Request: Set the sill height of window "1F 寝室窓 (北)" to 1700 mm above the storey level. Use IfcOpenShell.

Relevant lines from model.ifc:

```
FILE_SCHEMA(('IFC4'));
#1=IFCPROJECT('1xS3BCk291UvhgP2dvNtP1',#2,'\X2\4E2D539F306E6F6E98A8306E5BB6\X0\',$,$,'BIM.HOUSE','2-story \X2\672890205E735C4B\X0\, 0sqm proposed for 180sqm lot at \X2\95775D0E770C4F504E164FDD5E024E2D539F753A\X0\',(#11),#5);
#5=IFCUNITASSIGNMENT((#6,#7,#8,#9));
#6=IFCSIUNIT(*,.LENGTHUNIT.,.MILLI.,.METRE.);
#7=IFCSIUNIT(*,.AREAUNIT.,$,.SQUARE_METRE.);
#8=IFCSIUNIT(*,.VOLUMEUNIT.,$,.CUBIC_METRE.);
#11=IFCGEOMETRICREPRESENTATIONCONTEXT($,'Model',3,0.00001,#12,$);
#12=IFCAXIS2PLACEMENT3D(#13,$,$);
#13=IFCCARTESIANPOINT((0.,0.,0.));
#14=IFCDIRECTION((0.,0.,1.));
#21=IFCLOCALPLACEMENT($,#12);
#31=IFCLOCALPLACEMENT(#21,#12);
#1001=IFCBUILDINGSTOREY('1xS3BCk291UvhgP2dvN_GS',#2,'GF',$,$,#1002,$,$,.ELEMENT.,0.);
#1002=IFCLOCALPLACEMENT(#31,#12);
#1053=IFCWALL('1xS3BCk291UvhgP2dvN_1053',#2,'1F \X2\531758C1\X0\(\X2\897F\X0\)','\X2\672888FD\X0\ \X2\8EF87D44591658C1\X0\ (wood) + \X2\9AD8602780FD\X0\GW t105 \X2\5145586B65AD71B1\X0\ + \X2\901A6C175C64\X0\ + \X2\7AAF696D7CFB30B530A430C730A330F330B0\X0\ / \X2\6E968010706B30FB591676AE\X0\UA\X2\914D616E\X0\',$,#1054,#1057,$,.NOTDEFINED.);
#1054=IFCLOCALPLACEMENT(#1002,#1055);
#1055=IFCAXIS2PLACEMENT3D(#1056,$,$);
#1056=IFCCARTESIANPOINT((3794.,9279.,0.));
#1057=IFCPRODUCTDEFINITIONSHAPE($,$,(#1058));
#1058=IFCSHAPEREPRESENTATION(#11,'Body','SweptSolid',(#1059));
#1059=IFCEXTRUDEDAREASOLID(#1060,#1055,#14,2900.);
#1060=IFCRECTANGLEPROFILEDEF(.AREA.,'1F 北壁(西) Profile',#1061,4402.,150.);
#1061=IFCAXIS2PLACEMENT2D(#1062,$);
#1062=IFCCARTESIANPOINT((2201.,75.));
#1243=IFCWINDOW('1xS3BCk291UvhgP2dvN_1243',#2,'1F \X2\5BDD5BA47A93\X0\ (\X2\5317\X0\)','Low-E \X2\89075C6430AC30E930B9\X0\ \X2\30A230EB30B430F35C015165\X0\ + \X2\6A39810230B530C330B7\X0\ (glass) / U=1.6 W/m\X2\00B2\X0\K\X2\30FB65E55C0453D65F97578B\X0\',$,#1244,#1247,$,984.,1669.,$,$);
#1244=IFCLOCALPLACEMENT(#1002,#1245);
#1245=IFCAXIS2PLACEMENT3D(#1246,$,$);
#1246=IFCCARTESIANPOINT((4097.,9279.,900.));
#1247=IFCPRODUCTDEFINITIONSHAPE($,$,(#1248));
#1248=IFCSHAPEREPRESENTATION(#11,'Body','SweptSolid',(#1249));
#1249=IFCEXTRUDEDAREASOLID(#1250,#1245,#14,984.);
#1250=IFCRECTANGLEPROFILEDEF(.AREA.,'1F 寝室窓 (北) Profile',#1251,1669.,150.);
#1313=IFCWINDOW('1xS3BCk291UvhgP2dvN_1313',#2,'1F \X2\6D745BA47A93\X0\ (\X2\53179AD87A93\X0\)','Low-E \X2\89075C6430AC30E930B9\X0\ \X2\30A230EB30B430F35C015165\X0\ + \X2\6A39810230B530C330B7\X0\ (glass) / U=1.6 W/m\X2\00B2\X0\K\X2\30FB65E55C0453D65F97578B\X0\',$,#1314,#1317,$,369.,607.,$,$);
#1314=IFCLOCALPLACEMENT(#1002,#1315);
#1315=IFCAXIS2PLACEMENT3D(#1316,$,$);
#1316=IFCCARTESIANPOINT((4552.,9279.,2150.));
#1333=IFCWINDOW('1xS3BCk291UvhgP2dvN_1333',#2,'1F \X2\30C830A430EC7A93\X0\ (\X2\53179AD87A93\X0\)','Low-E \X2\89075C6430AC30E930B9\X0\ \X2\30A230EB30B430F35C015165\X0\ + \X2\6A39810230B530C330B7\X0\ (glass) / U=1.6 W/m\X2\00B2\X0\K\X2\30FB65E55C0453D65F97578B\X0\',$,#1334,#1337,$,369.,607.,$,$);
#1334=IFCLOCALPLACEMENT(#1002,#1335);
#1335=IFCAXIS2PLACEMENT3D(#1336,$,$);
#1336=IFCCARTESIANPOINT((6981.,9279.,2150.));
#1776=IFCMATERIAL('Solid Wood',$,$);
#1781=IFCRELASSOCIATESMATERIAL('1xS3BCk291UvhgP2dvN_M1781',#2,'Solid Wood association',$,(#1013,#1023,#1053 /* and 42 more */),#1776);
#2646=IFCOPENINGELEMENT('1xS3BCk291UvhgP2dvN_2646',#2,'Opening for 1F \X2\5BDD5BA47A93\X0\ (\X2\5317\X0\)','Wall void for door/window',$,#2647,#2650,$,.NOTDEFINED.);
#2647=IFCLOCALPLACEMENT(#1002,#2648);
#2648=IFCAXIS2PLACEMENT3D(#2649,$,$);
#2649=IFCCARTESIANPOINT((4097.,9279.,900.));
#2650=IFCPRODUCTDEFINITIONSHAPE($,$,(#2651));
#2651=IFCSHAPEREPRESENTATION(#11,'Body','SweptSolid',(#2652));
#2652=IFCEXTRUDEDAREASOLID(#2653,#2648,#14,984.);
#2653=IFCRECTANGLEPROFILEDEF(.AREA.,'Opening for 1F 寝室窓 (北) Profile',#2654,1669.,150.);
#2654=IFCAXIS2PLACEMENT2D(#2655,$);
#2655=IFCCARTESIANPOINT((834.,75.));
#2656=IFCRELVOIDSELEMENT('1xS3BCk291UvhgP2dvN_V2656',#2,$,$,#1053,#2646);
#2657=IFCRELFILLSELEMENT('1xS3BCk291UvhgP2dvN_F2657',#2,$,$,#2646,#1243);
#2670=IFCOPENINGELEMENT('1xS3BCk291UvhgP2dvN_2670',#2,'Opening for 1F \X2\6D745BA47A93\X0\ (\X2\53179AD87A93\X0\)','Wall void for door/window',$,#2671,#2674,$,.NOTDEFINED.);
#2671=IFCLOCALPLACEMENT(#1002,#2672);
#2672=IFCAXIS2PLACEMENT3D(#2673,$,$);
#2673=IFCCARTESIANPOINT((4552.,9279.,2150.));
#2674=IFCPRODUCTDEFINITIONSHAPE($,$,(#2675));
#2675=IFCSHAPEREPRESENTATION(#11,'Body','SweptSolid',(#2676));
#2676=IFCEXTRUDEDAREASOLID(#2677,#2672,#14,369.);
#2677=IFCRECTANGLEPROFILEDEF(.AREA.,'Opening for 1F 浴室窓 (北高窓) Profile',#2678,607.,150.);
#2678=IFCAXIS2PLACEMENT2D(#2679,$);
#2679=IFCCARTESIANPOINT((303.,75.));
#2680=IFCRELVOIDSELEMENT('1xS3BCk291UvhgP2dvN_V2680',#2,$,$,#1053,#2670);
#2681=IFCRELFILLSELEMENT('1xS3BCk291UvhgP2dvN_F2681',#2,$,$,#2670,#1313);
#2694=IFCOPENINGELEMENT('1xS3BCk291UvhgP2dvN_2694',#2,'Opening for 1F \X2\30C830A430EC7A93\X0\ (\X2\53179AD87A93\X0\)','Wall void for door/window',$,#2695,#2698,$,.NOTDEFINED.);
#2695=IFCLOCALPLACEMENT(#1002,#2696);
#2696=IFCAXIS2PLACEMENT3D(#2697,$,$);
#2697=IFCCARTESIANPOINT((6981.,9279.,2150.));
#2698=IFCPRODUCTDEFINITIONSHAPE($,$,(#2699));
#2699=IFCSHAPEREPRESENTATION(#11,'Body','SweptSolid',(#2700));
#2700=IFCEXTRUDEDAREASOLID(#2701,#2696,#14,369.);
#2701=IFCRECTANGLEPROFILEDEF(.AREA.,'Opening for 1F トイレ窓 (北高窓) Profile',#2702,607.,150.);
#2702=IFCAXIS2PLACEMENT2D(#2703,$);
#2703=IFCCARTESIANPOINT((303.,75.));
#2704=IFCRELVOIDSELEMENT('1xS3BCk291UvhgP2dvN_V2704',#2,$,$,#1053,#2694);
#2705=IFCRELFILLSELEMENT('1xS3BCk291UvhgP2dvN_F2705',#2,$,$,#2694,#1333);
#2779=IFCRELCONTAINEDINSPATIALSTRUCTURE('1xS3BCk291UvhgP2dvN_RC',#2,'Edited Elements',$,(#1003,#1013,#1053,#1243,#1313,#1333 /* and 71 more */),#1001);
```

```python
import numpy as np
import ifcopenshell
import ifcopenshell.api.geometry
import ifcopenshell.geom
import ifcopenshell.util.element
import ifcopenshell.util.placement
import ifcopenshell.util.shape
import ifcopenshell.util.unit

model = ifcopenshell.open("model.ifc")
unit_scale = ifcopenshell.util.unit.calculate_unit_scale(model)

window = model.by_id(1243)
opening = window.FillsVoids[0].RelatingOpeningElement
storey = ifcopenshell.util.element.get_container(window, ifc_class="IfcBuildingStorey")
level = ifcopenshell.util.placement.get_local_placement(storey.ObjectPlacement)[2, 3]

# The opening's origin need not be at the sill, so measure its lowest point.
shape = ifcopenshell.geom.create_shape(ifcopenshell.geom.settings(), opening)
bottom = ifcopenshell.util.shape.get_shape_bottom_elevation(shape, shape.geometry) / unit_scale
dz = level + 1.7 / unit_scale - bottom

shift = np.array([0.0, 0.0, dz])
# The window is not placed relative to its opening, so move both.
for product in (opening, window):
    matrix = ifcopenshell.util.placement.get_local_placement(product.ObjectPlacement)
    matrix[:3, 3] += shift
    ifcopenshell.api.geometry.edit_object_placement(model, product=product, matrix=matrix, is_si=False)

print(f"moved by {dz * unit_scale:+.3f} m")

model.write("model_updated.ifc")
```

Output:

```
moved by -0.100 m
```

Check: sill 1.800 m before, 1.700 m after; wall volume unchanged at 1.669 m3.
